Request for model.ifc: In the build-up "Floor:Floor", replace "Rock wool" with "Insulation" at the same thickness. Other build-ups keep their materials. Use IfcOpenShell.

First a look at what the model holds.

```python
import ifcopenshell
import ifcopenshell.util.element

model = ifcopenshell.open("model.ifc")
print(model.schema)
for layer_set in model.by_type("IfcMaterialLayerSet"):
    if layer_set.LayerSetName == "Floor:Floor":
        for layer in layer_set.MaterialLayers:
            print(layer.id(), layer.Material and layer.Material.Name, layer.LayerThickness, sep=" | ")
        print(len(ifcopenshell.util.element.get_elements_by_material(model, layer_set)), "elements and types use it")
print(sorted(m.Name for m in model.by_type("IfcMaterial") if m.Name)[:60])
```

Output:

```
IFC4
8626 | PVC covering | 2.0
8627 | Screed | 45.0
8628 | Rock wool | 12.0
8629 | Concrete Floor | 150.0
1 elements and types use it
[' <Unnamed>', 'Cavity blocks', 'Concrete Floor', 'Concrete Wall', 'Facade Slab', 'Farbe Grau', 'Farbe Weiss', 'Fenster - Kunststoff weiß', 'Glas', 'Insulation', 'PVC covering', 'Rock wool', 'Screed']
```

```python
import ifcopenshell
import ifcopenshell.api.material

model = ifcopenshell.open("model.ifc")

layer_set = next(s for s in model.by_type("IfcMaterialLayerSet") if s.LayerSetName == "Floor:Floor")
layer = next(l for l in layer_set.MaterialLayers if l.Material and l.Material.Name == "Rock wool")
material = next(m for m in model.by_type("IfcMaterial") if m.Name == "Insulation")

# Point this one layer at the other material; renaming the old one would change it everywhere.
ifcopenshell.api.material.edit_layer(model, layer=layer, attributes={}, material=material)

print([l.Material.Name if l.Material else None for l in layer_set.MaterialLayers])

model.write("model_v2.ifc")
```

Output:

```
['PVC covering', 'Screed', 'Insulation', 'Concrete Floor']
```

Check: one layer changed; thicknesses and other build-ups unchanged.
